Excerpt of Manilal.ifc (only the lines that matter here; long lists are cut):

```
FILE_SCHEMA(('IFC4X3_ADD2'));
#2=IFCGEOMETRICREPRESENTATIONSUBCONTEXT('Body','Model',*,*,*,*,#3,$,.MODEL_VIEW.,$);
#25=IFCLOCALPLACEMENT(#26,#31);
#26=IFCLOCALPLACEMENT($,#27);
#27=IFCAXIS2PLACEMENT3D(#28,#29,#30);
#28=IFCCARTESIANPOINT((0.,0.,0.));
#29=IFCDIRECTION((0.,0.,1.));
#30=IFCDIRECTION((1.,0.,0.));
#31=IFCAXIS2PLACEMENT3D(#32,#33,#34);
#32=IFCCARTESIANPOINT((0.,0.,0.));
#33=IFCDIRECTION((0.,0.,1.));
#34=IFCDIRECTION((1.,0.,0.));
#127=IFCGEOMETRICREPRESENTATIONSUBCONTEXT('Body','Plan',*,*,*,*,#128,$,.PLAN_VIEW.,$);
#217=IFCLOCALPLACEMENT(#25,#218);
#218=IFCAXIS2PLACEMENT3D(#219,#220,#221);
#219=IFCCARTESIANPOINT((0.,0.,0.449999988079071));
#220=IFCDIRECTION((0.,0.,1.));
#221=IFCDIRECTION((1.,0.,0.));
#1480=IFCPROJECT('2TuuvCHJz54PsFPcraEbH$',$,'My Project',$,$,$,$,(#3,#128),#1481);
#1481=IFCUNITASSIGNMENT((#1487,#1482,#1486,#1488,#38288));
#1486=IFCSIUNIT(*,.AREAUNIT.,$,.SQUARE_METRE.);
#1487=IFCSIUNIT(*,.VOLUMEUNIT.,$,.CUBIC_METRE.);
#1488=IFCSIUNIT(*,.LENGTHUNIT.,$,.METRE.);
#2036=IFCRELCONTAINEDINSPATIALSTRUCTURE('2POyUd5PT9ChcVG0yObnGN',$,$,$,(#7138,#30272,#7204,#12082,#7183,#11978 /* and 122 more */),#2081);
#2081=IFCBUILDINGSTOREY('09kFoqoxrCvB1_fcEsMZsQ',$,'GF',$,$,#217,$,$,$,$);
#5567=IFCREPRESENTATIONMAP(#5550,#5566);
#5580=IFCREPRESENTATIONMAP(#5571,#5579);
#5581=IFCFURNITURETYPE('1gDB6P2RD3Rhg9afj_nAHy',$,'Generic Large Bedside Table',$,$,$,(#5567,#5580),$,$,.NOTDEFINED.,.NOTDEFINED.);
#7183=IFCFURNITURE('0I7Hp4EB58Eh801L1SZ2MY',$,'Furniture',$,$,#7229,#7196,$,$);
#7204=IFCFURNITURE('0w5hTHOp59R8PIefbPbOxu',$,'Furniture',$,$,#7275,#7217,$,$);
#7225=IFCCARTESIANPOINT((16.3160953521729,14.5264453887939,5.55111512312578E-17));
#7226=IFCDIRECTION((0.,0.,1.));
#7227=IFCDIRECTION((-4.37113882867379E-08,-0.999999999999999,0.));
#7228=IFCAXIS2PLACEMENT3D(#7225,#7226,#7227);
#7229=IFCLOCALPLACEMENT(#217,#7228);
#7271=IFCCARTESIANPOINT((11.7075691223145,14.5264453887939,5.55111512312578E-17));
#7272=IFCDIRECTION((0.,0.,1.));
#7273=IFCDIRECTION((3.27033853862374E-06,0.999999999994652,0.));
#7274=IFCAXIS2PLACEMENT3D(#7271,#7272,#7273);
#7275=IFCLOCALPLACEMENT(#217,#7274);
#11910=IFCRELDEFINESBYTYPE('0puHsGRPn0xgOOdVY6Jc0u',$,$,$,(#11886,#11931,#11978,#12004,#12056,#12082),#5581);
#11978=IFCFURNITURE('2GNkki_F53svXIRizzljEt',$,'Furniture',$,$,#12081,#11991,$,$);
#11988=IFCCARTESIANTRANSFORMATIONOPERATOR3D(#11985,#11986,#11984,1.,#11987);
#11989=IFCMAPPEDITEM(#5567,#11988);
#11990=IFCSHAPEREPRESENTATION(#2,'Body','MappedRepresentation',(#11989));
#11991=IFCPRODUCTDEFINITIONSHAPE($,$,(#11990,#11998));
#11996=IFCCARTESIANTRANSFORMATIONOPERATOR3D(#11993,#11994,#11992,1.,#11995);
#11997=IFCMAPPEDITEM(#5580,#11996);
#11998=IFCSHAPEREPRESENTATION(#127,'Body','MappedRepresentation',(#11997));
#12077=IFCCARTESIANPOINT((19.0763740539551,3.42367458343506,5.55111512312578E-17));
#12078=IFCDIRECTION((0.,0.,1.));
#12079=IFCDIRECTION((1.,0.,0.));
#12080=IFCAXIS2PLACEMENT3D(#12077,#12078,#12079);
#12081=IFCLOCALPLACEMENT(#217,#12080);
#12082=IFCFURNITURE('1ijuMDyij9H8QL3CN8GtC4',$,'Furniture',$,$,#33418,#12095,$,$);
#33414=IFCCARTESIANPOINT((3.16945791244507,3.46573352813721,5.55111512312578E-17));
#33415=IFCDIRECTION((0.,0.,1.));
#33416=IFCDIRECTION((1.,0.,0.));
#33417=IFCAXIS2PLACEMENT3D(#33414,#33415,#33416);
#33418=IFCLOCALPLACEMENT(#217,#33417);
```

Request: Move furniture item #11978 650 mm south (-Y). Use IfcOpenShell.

```python
import ifcopenshell
import ifcopenshell.api.geometry
import ifcopenshell.util.placement
import ifcopenshell.util.unit

model = ifcopenshell.open("Manilal.ifc")
unit_scale = ifcopenshell.util.unit.calculate_unit_scale(model)

item = model.by_guid("2GNkki_F53svXIRizzljEt")
matrix = ifcopenshell.util.placement.get_local_placement(item.ObjectPlacement)
matrix[1, 3] -= 0.65 / unit_scale
ifcopenshell.api.geometry.edit_object_placement(model, product=item, matrix=matrix, is_si=False)

print(ifcopenshell.util.placement.get_local_placement(item.ObjectPlacement).round(3) + 0.0)

model.write("Manilal_updated.ifc")
```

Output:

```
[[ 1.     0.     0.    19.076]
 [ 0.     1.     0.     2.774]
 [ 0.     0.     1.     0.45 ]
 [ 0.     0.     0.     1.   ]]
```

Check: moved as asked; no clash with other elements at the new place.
